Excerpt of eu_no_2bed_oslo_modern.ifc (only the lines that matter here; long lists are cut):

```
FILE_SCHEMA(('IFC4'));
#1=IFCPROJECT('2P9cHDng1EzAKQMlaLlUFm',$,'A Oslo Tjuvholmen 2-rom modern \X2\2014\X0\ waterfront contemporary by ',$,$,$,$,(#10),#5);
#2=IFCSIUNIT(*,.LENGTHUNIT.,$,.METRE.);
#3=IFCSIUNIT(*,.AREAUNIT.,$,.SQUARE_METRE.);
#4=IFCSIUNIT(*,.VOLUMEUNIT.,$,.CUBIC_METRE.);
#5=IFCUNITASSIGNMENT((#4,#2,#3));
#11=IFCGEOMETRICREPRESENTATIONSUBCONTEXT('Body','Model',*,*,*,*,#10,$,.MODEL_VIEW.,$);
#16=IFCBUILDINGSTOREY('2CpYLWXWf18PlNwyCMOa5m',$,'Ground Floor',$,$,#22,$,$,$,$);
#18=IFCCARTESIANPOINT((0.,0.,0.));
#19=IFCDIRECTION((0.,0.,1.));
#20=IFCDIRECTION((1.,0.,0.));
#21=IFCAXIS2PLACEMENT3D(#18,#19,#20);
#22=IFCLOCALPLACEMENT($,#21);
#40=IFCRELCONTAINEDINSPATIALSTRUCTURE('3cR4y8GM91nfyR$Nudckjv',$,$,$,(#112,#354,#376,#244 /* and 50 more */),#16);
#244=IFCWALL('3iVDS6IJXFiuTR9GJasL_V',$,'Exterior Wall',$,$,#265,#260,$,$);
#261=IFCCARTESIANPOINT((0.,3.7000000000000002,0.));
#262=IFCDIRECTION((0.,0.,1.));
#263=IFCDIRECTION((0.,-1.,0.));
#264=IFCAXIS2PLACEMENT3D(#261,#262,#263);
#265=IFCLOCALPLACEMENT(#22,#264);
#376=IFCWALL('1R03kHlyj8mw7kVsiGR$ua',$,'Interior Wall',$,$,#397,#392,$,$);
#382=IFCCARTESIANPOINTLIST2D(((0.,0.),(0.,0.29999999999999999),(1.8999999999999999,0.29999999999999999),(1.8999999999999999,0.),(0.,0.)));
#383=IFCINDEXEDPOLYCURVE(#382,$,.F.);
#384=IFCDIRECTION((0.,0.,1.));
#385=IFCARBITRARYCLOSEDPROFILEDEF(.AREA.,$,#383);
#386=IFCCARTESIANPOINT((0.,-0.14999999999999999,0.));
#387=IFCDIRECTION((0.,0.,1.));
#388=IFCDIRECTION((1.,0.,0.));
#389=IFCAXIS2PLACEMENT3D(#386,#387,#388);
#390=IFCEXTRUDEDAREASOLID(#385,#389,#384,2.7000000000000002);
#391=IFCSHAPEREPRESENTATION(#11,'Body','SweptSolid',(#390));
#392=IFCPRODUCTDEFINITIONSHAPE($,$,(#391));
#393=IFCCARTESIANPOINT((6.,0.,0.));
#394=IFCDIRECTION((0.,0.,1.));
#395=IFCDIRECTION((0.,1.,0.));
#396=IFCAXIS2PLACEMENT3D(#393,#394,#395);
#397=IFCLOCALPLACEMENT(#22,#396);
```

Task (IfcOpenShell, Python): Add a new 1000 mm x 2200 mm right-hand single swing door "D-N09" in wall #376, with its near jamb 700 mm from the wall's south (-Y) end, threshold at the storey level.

```python
import numpy as np
import ifcopenshell
import ifcopenshell.api.feature
import ifcopenshell.api.geometry
import ifcopenshell.api.root
import ifcopenshell.api.spatial
import ifcopenshell.geom
import ifcopenshell.util.element
import ifcopenshell.util.placement
import ifcopenshell.util.representation
import ifcopenshell.util.shape
import ifcopenshell.util.unit

model = ifcopenshell.open("eu_no_2bed_oslo_modern.ifc")
unit_scale = ifcopenshell.util.unit.calculate_unit_scale(model)
settings = ifcopenshell.geom.settings()


def volume(element):
    """Net volume in cubic metres, openings subtracted."""
    shape = ifcopenshell.geom.create_shape(settings, element)
    return ifcopenshell.util.shape.get_volume(shape.geometry)


wall = model.by_guid("1R03kHlyj8mw7kVsiGR$ua")
storey = ifcopenshell.util.element.get_container(wall, ifc_class="IfcBuildingStorey")
context = ifcopenshell.util.representation.get_context(model, "Model", "Body", "MODEL_VIEW")
before = volume(wall)

width, height, from_end, sill = 1, 2.2, 0.7, 0.0  # metres

# The wall runs along its own X axis, and the end named is its -X end.
wall_shape = ifcopenshell.geom.create_shape(settings, wall)
x, y, z = ifcopenshell.util.shape.get_vertices(wall_shape.geometry).T
start = x.min() + from_end
face, thickness = float(y.min()), float(y.max() - y.min())
wall_matrix = ifcopenshell.util.placement.get_local_placement(wall.ObjectPlacement)
level = ifcopenshell.util.placement.get_local_placement(storey.ObjectPlacement)[2, 3]


def in_wall(x, y):
    """Placement at x, y metres in the wall's axes, at sill height."""
    matrix = wall_matrix.copy()
    matrix[:, 3] = wall_matrix @ np.array([x / unit_scale, y / unit_scale, 0.0, 1.0])
    matrix[2, 3] = level + sill / unit_scale
    return matrix


# Opening: a box that overshoots both wall faces by 50 mm.
opening = ifcopenshell.api.root.create_entity(model, ifc_class="IfcOpeningElement", predefined_type="OPENING")
box = ifcopenshell.api.geometry.add_wall_representation(
    model, context=context, length=width, height=height, thickness=thickness + 0.1
)
ifcopenshell.api.geometry.assign_representation(model, product=opening, representation=box)
ifcopenshell.api.geometry.edit_object_placement(model, product=opening, matrix=in_wall(start, face - 0.05), is_si=False)
ifcopenshell.api.feature.add_feature(model, feature=opening, element=wall)

door = ifcopenshell.api.root.create_entity(model, ifc_class="IfcDoor", name="D-N09", predefined_type="DOOR")
door.OverallWidth, door.OverallHeight = width / unit_scale, height / unit_scale
door.OperationType = "SINGLE_SWING_RIGHT"
body = ifcopenshell.api.geometry.add_door_representation(
    model,
    context=context,
    overall_width=door.OverallWidth,
    overall_height=door.OverallHeight,
    operation_type="SINGLE_SWING_RIGHT",
    lining_properties={"LiningDepth": thickness / unit_scale, "ThresholdDepth": thickness / unit_scale},
)
ifcopenshell.api.geometry.assign_representation(model, product=door, representation=body)
ifcopenshell.api.spatial.assign_container(model, products=[door], relating_structure=storey)
ifcopenshell.api.feature.add_filling(model, opening=opening, element=door)

# The lining spans the wall, so the door starts at the wall face.
ifcopenshell.api.geometry.edit_object_placement(model, product=door, matrix=in_wall(start, face), is_si=False)

after = volume(wall)

print(f"wall volume {before:.3f} -> {after:.3f} m3")

model.write("eu_no_2bed_oslo_modern-out.ifc")
```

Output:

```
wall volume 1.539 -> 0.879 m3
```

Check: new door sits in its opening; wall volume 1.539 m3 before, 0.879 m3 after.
